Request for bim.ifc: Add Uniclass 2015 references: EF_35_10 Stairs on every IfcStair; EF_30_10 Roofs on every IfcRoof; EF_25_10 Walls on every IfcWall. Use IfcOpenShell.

First a look at what the model holds.

```python
import ifcopenshell

model = ifcopenshell.open("bim.ifc")
print(model.schema)
print("classifications:", [c.Name for c in model.by_type("IfcClassification")])
for ifc_class in ("IfcDoor", "IfcRoof", "IfcStair", "IfcWall", "IfcWindow"):
    print(ifc_class, len(model.by_type(ifc_class)))
```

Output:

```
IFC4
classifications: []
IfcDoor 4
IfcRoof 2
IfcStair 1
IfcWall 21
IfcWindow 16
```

```python
import ifcopenshell
import ifcopenshell.api.classification

model = ifcopenshell.open("bim.ifc")

system = ifcopenshell.api.classification.add_classification(model, classification="Uniclass 2015")

codes = {
    "IfcStair": ("EF_35_10", "Stairs"),
    "IfcRoof": ("EF_30_10", "Roofs"),
    "IfcWall": ("EF_25_10", "Walls"),
}
for ifc_class, (code, name) in codes.items():
    products = model.by_type(ifc_class)
    ifcopenshell.api.classification.add_reference(
        model, products=products, classification=system, identification=code, name=name
    )
    print(code, len(products))

model.write("bim-out.ifc")
```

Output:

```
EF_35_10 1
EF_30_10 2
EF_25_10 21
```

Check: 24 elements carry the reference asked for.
